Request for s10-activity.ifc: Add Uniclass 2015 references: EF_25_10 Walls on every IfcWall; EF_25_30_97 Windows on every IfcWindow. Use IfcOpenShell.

First a look at what the model holds.

```python
import ifcopenshell

model = ifcopenshell.open("s10-activity.ifc")
print(model.schema)
print("classifications:", [c.Name for c in model.by_type("IfcClassification")])
for ifc_class in ("IfcDoor", "IfcRoof", "IfcStair", "IfcWall", "IfcWindow"):
    print(ifc_class, len(model.by_type(ifc_class)))
```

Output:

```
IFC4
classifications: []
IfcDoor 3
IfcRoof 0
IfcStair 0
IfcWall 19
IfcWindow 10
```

```python
import ifcopenshell
import ifcopenshell.api.classification

model = ifcopenshell.open("s10-activity.ifc")

system = ifcopenshell.api.classification.add_classification(model, classification="Uniclass 2015")

codes = {
    "IfcWall": ("EF_25_10", "Walls"),
    "IfcWindow": ("EF_25_30_97", "Windows"),
}
for ifc_class, (code, name) in codes.items():
    products = model.by_type(ifc_class)
    ifcopenshell.api.classification.add_reference(
        model, products=products, classification=system, identification=code, name=name
    )
    print(code, len(products))

model.write("s10-activity_rev.ifc")
```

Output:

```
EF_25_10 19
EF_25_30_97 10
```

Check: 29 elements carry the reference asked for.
